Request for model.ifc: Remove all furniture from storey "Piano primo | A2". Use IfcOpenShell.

First a look at what the model holds.

```python
import ifcopenshell
import ifcopenshell.util.element

model = ifcopenshell.open("model.ifc")
print(model.schema)
storey = next(s for s in model.by_type("IfcBuildingStorey") if s.Name == "Piano primo | A2")
furniture = [e for e in ifcopenshell.util.element.get_decomposition(storey) if e.is_a("IfcFurnishingElement")]
seen = {}
for e in furniture:
    element_type = ifcopenshell.util.element.get_type(e)
    name = element_type.Name if element_type not in (None, e) else None
    seen[name] = seen.get(name, 0) + 1
for name, count in sorted(seen.items(), key=str):
    print(count, "x", name)
```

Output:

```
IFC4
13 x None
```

```python
import ifcopenshell
import ifcopenshell.api.root
import ifcopenshell.util.element

model = ifcopenshell.open("model.ifc")

storey = next(s for s in model.by_type("IfcBuildingStorey") if s.Name == "Piano primo | A2")
furniture = [e for e in ifcopenshell.util.element.get_decomposition(storey) if e.is_a("IfcFurnishingElement")]

for e in furniture:
    ifcopenshell.api.root.remove_product(model, product=e)
print(len(furniture), "removed")

model.write("model_rev.ifc")
```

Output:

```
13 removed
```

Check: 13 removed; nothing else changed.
